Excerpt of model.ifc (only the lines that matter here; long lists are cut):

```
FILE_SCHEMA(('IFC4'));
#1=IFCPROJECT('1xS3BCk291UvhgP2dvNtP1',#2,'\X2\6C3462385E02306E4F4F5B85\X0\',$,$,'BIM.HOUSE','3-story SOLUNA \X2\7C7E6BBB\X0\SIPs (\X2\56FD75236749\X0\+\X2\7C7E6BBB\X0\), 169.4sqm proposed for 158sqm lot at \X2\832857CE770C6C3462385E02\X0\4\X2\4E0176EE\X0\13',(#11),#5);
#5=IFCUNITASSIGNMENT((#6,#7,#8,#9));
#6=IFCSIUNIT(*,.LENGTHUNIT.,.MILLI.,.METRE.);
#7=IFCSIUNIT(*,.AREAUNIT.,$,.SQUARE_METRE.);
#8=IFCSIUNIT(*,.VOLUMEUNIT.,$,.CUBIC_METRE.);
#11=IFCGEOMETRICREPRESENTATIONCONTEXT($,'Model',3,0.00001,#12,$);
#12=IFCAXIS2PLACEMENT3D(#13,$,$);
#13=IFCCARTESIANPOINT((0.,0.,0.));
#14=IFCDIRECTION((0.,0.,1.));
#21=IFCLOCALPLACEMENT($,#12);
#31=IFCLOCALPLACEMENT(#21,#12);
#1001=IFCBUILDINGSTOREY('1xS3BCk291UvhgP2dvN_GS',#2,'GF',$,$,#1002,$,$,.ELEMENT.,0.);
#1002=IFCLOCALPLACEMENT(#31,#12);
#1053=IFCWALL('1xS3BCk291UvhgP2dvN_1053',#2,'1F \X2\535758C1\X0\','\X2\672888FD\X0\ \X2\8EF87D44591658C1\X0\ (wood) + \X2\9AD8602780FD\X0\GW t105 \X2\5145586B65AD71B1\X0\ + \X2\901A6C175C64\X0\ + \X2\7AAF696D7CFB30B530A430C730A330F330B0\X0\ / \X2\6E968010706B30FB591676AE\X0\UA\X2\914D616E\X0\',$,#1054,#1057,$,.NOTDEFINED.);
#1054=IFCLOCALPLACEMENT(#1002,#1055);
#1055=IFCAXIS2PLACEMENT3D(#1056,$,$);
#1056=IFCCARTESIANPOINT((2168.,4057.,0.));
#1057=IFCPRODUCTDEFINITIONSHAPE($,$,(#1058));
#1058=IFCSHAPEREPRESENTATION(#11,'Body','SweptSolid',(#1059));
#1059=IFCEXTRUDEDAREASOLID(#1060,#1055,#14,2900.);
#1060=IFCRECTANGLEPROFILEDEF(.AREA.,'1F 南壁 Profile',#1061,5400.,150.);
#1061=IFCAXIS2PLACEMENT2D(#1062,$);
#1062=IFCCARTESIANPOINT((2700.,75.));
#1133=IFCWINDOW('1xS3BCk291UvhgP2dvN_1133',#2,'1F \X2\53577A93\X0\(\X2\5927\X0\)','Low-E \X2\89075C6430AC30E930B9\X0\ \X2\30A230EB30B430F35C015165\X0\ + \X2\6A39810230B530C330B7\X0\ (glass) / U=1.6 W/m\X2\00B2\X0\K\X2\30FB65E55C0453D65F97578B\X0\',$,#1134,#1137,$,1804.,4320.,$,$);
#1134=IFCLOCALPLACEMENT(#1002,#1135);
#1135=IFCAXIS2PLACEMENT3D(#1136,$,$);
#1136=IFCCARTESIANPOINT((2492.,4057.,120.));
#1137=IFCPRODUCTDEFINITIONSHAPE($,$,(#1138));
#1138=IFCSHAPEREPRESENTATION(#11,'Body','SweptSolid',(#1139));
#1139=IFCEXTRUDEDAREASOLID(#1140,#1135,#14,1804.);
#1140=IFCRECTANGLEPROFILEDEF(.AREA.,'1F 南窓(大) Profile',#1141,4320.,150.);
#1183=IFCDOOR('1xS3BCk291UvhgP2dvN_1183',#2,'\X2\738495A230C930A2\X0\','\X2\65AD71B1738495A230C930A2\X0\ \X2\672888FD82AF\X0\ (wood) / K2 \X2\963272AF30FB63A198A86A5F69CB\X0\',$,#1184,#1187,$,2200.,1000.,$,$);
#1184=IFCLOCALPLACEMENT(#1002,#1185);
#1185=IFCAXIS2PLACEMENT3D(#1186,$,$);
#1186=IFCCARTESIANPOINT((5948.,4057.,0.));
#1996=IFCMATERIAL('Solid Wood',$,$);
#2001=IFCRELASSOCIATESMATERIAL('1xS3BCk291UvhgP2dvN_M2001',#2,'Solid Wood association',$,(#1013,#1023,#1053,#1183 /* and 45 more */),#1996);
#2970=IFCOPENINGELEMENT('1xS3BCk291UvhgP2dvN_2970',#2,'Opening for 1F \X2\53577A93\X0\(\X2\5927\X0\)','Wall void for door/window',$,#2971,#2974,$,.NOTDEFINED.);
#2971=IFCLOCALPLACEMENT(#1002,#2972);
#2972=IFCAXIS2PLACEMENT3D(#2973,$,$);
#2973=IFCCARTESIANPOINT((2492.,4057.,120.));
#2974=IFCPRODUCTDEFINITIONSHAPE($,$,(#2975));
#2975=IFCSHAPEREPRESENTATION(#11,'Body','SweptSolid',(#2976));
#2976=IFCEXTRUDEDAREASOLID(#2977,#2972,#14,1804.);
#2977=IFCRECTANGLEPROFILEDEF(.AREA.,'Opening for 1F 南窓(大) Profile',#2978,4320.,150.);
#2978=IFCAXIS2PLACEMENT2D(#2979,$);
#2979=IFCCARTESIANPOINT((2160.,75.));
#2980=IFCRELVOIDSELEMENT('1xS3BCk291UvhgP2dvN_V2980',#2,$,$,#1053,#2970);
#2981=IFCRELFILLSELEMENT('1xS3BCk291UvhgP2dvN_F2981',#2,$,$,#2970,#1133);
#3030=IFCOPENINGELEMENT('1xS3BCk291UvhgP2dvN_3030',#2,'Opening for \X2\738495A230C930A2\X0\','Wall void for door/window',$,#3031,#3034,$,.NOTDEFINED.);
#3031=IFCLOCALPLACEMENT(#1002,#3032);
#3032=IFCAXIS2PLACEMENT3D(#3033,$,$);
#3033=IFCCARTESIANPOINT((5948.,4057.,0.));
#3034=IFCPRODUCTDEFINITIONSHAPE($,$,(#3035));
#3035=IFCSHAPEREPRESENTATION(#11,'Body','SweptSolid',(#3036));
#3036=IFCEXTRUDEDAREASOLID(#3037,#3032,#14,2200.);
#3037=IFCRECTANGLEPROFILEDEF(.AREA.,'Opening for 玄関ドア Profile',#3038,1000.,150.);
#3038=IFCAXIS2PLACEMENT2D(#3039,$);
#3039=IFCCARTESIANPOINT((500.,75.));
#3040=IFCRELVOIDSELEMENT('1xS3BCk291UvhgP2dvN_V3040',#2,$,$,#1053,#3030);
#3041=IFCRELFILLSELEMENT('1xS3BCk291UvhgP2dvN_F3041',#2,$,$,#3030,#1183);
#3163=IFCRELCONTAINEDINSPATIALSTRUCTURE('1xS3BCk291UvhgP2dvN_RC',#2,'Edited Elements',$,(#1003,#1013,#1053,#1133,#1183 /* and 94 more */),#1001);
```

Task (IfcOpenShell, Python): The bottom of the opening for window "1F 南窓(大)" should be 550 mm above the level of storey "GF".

```python
import numpy as np
import ifcopenshell
import ifcopenshell.api.geometry
import ifcopenshell.geom
import ifcopenshell.util.element
import ifcopenshell.util.placement
import ifcopenshell.util.shape
import ifcopenshell.util.unit

model = ifcopenshell.open("model.ifc")
unit_scale = ifcopenshell.util.unit.calculate_unit_scale(model)

window = model.by_id(1133)
opening = window.FillsVoids[0].RelatingOpeningElement
storey = ifcopenshell.util.element.get_container(window, ifc_class="IfcBuildingStorey")
level = ifcopenshell.util.placement.get_local_placement(storey.ObjectPlacement)[2, 3]

# The opening's origin need not be at the sill, so measure its lowest point.
shape = ifcopenshell.geom.create_shape(ifcopenshell.geom.settings(), opening)
bottom = ifcopenshell.util.shape.get_shape_bottom_elevation(shape, shape.geometry) / unit_scale
dz = level + 550.0 - bottom

shift = np.array([0.0, 0.0, dz])
# The window is not placed relative to its opening, so move both.
for product in (opening, window):
    matrix = ifcopenshell.util.placement.get_local_placement(product.ObjectPlacement)
    matrix[:3, 3] += shift
    ifcopenshell.api.geometry.edit_object_placement(model, product=product, matrix=matrix, is_si=False)

print(f"moved by {dz * unit_scale:+.3f} m")

model.write("model-out.ifc")
```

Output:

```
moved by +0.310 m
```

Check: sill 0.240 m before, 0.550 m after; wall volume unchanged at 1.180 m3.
